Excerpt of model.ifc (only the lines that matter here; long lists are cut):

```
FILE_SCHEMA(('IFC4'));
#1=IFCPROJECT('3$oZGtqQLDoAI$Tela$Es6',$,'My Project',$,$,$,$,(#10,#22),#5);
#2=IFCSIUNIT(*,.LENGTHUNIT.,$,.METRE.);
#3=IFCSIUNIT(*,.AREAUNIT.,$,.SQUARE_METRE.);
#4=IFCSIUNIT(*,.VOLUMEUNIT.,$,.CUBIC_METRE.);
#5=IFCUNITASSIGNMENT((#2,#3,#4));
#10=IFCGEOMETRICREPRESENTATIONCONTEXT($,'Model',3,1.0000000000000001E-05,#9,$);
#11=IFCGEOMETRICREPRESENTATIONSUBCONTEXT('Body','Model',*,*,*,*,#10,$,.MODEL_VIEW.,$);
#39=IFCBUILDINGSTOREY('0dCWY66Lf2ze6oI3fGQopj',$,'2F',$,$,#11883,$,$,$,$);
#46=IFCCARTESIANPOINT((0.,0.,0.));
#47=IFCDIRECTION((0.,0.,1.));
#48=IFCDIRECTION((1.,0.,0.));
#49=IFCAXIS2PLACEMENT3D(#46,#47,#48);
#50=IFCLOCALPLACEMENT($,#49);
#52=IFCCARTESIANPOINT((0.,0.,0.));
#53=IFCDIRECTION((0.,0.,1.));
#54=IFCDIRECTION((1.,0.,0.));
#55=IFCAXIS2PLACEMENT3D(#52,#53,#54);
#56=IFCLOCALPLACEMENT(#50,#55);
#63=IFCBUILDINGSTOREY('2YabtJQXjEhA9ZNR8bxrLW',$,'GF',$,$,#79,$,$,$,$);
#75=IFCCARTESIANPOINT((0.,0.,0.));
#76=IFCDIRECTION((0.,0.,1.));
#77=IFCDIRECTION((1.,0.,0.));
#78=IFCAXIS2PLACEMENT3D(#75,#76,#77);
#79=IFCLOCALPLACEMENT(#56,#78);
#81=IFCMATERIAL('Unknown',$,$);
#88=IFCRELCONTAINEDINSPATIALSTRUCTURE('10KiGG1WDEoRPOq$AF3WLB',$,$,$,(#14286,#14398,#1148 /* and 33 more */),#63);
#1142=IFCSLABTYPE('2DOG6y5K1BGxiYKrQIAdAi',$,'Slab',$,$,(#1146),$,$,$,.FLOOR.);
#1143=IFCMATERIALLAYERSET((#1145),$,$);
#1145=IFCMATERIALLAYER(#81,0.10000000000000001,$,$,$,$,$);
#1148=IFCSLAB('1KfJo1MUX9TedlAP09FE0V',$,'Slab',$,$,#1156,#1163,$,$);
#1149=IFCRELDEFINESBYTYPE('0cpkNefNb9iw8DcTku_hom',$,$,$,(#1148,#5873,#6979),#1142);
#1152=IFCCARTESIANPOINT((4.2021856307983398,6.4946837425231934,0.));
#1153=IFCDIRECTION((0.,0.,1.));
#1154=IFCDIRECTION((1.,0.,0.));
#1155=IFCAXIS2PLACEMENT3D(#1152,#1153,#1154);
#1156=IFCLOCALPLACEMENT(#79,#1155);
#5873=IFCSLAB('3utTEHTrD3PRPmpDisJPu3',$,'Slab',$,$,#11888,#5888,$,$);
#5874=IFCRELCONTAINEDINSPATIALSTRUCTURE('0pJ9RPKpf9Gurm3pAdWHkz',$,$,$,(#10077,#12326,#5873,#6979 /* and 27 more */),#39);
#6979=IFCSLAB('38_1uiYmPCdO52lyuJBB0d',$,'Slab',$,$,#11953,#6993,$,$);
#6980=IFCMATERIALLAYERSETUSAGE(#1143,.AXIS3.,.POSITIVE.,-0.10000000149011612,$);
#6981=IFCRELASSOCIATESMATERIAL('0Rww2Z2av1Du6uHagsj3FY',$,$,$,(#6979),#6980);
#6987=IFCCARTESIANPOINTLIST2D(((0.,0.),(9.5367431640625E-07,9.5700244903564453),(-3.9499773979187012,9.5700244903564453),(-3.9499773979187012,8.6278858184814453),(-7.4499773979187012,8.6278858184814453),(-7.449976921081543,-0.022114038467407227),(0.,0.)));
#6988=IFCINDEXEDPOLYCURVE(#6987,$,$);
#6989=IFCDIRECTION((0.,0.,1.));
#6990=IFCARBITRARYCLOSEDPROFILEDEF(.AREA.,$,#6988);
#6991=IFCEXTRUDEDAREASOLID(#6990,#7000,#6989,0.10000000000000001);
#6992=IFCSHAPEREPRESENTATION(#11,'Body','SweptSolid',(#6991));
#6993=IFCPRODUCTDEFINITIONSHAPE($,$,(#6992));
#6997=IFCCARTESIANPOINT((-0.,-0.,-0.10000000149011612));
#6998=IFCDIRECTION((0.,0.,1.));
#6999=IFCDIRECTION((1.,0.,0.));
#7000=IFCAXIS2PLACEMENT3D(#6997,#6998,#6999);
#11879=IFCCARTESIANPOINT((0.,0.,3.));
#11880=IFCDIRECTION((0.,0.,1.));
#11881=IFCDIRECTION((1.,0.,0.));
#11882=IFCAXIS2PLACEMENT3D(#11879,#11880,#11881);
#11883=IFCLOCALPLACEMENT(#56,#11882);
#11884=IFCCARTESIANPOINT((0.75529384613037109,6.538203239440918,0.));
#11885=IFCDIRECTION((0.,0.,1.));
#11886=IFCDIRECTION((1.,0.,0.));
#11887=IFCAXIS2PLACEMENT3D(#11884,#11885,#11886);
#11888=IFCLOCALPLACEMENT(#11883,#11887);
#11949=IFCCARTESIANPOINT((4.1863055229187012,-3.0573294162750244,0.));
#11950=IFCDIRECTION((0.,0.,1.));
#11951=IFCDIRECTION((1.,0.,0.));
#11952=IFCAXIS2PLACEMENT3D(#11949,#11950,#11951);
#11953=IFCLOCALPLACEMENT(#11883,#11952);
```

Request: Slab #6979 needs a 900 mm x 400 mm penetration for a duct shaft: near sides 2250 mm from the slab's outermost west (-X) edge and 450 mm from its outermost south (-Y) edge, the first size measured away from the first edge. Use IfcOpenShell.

```python
import numpy as np
import ifcopenshell
import ifcopenshell.api.feature
import ifcopenshell.api.geometry
import ifcopenshell.api.root
import ifcopenshell.geom
import ifcopenshell.util.placement
import ifcopenshell.util.representation
import ifcopenshell.util.shape
import ifcopenshell.util.unit

model = ifcopenshell.open("model.ifc")
unit_scale = ifcopenshell.util.unit.calculate_unit_scale(model)
settings = ifcopenshell.geom.settings()


def volume(element):
    """Net volume in cubic metres, openings subtracted."""
    shape = ifcopenshell.geom.create_shape(settings, element)
    return ifcopenshell.util.shape.get_volume(shape.geometry)


slab = model.by_guid("38_1uiYmPCdO52lyuJBB0d")
before = volume(slab)

# Extent in the slab's own axes, in metres. The edges named are its -X and -Y sides.
slab_shape = ifcopenshell.geom.create_shape(settings, slab)
vertices = ifcopenshell.util.shape.get_vertices(slab_shape.geometry)
x_min, y_min, bottom = vertices.min(axis=0)
top = vertices[:, 2].max()

opening = ifcopenshell.api.root.create_entity(model, ifc_class="IfcOpeningElement", name="Duct shaft opening", predefined_type="OPENING")
context = ifcopenshell.util.representation.get_context(model, "Model", "Body", "MODEL_VIEW")
width, depth = 0.9, 0.4
outline = [(0.0, 0.0), (width, 0.0), (width, depth), (0.0, depth), (0.0, 0.0)]
# Overshoot both faces by 50 mm so the cut is clean.
shape = ifcopenshell.api.geometry.add_slab_representation(
    model, context=context, depth=top - bottom + 0.1, polyline=outline
)
ifcopenshell.api.geometry.assign_representation(model, product=opening, representation=shape)

matrix = ifcopenshell.util.placement.get_local_placement(slab.ObjectPlacement)
matrix[:, 3] = matrix @ np.append(np.array([x_min + 2.25, y_min + 0.45, bottom - 0.05]) / unit_scale, 1.0)
ifcopenshell.api.geometry.edit_object_placement(model, product=opening, matrix=matrix, is_si=False)
ifcopenshell.api.feature.add_feature(model, feature=opening, element=slab)

after = volume(slab)

print(f"slab volume {before:.3f} -> {after:.3f} m3")

model.write("model_updated.ifc")
```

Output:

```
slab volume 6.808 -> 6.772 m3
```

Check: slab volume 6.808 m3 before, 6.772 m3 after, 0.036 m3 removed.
